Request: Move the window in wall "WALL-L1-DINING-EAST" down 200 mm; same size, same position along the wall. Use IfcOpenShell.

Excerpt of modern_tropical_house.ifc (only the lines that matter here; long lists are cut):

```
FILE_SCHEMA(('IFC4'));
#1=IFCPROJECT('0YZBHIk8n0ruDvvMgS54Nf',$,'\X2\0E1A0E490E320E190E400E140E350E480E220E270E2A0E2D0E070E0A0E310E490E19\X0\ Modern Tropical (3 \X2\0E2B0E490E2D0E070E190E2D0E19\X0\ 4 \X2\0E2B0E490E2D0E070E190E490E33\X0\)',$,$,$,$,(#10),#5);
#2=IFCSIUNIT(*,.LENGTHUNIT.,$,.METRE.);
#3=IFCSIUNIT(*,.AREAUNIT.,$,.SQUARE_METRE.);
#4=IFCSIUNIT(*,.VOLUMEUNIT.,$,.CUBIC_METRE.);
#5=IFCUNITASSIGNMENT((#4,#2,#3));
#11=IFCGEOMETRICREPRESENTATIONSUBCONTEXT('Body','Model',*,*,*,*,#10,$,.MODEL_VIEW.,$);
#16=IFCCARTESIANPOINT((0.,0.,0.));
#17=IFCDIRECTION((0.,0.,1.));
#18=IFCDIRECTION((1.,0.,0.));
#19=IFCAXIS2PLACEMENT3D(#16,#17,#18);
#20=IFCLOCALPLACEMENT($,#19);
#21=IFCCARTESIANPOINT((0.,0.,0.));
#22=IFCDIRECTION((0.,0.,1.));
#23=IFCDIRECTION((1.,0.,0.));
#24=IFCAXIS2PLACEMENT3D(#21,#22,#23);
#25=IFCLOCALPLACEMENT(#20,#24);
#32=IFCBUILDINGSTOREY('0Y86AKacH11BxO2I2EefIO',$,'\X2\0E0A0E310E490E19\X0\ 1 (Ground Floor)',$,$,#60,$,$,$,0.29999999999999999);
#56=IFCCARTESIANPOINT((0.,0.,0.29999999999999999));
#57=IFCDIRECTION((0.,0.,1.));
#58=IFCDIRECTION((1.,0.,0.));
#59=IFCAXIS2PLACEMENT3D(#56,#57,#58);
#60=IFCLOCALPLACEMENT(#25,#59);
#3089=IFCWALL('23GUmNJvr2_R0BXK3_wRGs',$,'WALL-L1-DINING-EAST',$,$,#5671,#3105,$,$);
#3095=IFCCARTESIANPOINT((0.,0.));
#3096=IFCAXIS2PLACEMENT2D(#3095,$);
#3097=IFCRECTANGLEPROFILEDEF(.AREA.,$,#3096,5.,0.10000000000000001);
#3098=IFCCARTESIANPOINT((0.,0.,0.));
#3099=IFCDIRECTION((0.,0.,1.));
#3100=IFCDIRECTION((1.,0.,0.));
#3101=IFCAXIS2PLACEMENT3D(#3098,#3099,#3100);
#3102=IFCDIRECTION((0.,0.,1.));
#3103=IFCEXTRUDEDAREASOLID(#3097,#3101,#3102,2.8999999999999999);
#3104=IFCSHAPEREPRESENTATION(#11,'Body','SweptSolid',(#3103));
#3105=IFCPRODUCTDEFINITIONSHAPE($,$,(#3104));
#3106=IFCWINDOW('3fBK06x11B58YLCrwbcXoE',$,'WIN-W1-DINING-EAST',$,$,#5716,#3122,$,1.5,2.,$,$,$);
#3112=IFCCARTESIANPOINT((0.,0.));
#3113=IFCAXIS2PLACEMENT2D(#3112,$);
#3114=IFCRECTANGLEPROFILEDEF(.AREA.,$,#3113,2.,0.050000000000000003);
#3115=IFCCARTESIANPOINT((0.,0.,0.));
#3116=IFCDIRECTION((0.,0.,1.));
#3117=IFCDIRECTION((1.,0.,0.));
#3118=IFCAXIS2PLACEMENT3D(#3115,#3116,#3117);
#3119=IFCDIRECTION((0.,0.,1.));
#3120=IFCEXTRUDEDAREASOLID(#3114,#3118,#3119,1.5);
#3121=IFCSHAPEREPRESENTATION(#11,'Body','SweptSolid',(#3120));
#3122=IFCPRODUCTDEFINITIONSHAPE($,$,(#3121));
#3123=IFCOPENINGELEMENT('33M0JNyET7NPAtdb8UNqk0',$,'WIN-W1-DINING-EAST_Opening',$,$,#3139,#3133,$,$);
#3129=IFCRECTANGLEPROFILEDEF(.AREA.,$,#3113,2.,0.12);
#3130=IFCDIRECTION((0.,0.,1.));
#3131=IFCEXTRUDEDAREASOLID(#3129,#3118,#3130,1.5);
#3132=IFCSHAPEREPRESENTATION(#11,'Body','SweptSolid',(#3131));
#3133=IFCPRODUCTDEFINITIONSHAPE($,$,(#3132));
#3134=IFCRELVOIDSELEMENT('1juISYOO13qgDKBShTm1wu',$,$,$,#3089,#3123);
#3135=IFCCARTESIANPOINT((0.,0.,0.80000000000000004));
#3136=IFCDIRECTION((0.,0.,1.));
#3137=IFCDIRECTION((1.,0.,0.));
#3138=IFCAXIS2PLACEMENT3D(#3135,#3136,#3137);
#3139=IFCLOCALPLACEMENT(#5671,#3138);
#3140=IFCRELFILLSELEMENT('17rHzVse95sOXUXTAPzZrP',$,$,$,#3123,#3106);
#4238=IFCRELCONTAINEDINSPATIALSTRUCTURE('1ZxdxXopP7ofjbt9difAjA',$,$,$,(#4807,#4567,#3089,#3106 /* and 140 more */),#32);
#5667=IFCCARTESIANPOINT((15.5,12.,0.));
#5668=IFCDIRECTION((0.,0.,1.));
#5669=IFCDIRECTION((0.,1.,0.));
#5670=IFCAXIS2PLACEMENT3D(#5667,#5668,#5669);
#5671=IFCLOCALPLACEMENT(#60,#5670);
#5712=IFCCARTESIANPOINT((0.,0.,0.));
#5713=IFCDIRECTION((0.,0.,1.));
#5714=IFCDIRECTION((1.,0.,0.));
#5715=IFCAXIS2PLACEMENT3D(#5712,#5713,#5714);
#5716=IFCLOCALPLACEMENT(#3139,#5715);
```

```python
import numpy as np
import ifcopenshell
import ifcopenshell.api.geometry
import ifcopenshell.util.placement
import ifcopenshell.util.unit

model = ifcopenshell.open("modern_tropical_house.ifc")
unit_scale = ifcopenshell.util.unit.calculate_unit_scale(model)

window = model.by_id(3106)
opening = window.FillsVoids[0].RelatingOpeningElement
dz = -0.2 / unit_scale

shift = np.array([0.0, 0.0, dz])
# The window is placed relative to its opening, so it follows when the opening moves.
matrix = ifcopenshell.util.placement.get_local_placement(opening.ObjectPlacement)
matrix[:3, 3] += shift
ifcopenshell.api.geometry.edit_object_placement(
    model, product=opening, matrix=matrix, is_si=False, should_transform_children=True
)

print(f"moved by {dz * unit_scale:+.3f} m")

model.write("modern_tropical_house_edited.ifc")
```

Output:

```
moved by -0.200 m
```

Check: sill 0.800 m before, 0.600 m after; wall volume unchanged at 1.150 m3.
